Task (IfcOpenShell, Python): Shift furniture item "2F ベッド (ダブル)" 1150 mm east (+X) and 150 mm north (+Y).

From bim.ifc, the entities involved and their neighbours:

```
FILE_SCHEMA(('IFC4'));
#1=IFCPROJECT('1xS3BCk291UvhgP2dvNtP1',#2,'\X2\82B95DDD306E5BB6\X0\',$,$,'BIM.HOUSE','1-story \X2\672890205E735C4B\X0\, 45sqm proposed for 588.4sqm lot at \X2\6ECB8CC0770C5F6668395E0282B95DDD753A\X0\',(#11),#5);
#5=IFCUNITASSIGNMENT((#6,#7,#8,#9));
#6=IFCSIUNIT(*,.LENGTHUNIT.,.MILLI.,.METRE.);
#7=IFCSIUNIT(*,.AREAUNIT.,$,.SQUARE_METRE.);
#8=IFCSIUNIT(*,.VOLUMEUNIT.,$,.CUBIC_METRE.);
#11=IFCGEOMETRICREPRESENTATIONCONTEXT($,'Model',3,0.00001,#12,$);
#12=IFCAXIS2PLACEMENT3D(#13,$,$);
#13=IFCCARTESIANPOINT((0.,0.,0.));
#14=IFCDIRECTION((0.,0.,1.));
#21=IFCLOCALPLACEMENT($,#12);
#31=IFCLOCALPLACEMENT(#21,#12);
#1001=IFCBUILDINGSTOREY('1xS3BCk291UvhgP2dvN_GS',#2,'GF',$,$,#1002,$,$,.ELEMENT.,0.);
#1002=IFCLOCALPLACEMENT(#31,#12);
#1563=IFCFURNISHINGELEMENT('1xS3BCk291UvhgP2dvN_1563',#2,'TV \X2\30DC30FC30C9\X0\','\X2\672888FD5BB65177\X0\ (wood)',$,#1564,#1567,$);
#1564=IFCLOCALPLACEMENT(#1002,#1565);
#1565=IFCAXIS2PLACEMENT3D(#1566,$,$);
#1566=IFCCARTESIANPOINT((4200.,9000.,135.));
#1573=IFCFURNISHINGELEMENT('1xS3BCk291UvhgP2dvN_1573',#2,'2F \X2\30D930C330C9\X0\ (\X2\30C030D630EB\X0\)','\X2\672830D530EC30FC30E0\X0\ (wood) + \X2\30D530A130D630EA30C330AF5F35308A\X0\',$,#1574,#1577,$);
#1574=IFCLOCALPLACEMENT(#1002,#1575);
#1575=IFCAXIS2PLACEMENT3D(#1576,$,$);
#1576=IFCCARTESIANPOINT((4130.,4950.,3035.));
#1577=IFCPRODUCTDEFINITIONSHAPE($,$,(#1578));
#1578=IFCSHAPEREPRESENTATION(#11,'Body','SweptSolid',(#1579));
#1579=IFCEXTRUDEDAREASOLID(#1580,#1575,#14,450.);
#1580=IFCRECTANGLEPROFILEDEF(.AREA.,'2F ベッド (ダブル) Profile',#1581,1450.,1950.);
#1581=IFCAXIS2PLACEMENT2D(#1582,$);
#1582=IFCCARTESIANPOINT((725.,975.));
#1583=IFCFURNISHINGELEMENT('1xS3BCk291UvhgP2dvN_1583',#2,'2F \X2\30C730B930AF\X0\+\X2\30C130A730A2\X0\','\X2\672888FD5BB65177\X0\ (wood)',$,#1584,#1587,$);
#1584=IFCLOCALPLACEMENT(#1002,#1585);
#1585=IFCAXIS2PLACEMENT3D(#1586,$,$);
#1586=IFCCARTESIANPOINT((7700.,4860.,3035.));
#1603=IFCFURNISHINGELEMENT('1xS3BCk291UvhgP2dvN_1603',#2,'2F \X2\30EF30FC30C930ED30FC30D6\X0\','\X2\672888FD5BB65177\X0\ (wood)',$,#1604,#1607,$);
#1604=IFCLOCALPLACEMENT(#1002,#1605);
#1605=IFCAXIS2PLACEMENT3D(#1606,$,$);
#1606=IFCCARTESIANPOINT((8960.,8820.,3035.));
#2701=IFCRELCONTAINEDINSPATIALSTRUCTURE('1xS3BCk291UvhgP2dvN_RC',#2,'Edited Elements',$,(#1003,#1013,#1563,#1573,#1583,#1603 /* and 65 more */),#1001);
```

```python
import ifcopenshell
import ifcopenshell.api.geometry
import ifcopenshell.util.placement
import ifcopenshell.util.unit

model = ifcopenshell.open("bim.ifc")
unit_scale = ifcopenshell.util.unit.calculate_unit_scale(model)

item = model.by_id(1573)
matrix = ifcopenshell.util.placement.get_local_placement(item.ObjectPlacement)
matrix[0, 3] += 1.15 / unit_scale
matrix[1, 3] += 0.15 / unit_scale
ifcopenshell.api.geometry.edit_object_placement(model, product=item, matrix=matrix, is_si=False)

print(ifcopenshell.util.placement.get_local_placement(item.ObjectPlacement).round(3) + 0.0)

model.write("bim-out.ifc")
```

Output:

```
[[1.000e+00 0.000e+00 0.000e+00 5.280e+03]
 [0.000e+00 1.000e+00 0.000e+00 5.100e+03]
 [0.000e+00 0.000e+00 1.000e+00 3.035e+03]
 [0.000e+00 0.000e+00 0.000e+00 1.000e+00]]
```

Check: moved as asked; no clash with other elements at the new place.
